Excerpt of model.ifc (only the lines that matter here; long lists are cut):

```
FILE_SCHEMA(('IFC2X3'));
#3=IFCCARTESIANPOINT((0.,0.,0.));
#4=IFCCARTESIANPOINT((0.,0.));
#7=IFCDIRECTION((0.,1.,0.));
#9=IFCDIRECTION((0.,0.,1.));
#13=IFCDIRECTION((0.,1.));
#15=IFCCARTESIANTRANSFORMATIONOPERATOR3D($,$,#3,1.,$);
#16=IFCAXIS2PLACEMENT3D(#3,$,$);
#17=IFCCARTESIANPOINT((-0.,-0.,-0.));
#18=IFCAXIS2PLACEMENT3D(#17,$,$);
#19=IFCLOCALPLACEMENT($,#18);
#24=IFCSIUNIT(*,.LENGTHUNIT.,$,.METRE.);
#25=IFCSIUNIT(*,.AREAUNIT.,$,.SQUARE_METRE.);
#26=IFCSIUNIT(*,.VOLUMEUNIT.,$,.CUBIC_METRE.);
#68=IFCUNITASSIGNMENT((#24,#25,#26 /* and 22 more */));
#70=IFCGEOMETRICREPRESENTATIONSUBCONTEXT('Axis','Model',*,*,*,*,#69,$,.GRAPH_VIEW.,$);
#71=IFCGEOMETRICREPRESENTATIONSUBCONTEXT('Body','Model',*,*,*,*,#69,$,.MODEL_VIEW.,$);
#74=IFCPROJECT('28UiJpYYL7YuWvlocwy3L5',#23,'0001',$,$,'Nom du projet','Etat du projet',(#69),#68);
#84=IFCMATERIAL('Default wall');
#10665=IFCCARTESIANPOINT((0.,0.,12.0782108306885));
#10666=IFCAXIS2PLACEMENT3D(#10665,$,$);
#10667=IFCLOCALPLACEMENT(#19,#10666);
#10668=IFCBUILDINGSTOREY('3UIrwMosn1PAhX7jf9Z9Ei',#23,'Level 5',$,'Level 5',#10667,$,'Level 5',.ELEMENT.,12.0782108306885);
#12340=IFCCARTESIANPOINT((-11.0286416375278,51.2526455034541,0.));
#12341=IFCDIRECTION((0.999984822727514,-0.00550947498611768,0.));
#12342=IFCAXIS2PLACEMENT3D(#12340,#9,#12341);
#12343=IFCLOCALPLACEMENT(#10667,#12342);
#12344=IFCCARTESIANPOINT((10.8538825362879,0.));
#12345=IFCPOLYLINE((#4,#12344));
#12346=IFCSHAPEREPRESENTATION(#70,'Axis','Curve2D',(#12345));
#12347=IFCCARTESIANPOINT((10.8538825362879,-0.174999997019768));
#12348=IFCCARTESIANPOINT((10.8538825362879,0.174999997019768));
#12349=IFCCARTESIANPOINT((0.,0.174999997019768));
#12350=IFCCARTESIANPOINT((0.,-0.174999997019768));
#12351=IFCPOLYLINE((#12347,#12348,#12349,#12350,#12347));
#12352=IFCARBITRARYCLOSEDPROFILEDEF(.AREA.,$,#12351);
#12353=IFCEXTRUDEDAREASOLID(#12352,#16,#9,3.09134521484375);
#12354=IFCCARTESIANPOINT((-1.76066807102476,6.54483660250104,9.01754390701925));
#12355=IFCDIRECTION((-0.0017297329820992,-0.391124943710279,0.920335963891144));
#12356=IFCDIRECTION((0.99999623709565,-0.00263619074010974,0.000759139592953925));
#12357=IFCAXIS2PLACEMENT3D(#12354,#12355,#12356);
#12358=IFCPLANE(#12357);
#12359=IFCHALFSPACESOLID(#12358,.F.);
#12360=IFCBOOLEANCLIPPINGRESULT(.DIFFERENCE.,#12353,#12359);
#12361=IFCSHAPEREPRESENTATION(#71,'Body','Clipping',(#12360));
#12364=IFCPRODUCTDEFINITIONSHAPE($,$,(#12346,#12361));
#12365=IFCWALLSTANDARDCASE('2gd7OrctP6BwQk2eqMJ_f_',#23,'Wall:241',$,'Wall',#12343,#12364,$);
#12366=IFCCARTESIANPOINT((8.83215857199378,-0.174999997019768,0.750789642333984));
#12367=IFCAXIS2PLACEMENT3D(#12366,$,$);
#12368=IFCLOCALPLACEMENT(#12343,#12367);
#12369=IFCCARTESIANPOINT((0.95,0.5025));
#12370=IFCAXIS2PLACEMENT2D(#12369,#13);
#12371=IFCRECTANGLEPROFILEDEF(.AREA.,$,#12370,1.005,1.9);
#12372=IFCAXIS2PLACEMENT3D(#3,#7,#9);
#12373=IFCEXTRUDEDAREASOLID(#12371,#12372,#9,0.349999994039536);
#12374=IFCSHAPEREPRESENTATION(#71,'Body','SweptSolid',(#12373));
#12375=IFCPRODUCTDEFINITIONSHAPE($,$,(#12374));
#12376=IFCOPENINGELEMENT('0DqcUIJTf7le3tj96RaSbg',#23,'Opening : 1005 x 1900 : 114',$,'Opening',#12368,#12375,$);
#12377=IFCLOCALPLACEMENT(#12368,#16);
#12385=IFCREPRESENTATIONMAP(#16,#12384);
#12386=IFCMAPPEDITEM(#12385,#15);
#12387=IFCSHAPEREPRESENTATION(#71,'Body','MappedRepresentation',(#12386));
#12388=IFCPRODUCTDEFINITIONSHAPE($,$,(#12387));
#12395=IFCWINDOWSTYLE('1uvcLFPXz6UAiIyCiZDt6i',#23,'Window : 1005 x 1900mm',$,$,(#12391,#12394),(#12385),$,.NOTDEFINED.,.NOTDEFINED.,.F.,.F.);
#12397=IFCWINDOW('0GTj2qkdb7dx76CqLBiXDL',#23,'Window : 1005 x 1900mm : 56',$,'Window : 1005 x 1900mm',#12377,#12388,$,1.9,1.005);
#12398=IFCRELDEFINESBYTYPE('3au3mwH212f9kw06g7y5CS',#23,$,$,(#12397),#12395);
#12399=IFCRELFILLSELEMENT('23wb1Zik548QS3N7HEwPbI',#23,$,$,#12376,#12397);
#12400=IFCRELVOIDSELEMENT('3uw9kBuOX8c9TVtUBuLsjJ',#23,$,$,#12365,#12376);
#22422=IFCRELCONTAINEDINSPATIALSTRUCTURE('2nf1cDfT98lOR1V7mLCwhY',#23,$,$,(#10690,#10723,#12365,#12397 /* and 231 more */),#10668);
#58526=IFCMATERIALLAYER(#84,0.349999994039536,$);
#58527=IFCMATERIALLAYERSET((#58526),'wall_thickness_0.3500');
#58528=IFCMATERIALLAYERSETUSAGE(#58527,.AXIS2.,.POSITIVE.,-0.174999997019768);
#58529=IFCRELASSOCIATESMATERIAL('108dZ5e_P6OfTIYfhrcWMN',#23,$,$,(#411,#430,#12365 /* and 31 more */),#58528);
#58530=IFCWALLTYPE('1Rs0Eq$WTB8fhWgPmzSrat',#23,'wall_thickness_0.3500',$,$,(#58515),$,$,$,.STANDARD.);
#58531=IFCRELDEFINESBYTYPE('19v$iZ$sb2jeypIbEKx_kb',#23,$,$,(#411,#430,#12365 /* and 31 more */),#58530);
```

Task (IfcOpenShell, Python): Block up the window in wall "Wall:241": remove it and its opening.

```python
import ifcopenshell
import ifcopenshell.api.feature
import ifcopenshell.api.root
import ifcopenshell.geom
import ifcopenshell.util.shape

model = ifcopenshell.open("model.ifc")
settings = ifcopenshell.geom.settings()


def volume(element):
    """Net volume in cubic metres, openings subtracted."""
    shape = ifcopenshell.geom.create_shape(settings, element)
    return ifcopenshell.util.shape.get_volume(shape.geometry)


window = model.by_id(12397)
opening = window.FillsVoids[0].RelatingOpeningElement
wall = opening.VoidsElements[0].RelatingBuildingElement
before = volume(wall)

ifcopenshell.api.root.remove_product(model, product=window)
ifcopenshell.api.feature.remove_feature(model, feature=opening)

after = volume(wall)

print(f"wall volume {before:.3f} -> {after:.3f} m3")

model.write("model_edited.ifc")
```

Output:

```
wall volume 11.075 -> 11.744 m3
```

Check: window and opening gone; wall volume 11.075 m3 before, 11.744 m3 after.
